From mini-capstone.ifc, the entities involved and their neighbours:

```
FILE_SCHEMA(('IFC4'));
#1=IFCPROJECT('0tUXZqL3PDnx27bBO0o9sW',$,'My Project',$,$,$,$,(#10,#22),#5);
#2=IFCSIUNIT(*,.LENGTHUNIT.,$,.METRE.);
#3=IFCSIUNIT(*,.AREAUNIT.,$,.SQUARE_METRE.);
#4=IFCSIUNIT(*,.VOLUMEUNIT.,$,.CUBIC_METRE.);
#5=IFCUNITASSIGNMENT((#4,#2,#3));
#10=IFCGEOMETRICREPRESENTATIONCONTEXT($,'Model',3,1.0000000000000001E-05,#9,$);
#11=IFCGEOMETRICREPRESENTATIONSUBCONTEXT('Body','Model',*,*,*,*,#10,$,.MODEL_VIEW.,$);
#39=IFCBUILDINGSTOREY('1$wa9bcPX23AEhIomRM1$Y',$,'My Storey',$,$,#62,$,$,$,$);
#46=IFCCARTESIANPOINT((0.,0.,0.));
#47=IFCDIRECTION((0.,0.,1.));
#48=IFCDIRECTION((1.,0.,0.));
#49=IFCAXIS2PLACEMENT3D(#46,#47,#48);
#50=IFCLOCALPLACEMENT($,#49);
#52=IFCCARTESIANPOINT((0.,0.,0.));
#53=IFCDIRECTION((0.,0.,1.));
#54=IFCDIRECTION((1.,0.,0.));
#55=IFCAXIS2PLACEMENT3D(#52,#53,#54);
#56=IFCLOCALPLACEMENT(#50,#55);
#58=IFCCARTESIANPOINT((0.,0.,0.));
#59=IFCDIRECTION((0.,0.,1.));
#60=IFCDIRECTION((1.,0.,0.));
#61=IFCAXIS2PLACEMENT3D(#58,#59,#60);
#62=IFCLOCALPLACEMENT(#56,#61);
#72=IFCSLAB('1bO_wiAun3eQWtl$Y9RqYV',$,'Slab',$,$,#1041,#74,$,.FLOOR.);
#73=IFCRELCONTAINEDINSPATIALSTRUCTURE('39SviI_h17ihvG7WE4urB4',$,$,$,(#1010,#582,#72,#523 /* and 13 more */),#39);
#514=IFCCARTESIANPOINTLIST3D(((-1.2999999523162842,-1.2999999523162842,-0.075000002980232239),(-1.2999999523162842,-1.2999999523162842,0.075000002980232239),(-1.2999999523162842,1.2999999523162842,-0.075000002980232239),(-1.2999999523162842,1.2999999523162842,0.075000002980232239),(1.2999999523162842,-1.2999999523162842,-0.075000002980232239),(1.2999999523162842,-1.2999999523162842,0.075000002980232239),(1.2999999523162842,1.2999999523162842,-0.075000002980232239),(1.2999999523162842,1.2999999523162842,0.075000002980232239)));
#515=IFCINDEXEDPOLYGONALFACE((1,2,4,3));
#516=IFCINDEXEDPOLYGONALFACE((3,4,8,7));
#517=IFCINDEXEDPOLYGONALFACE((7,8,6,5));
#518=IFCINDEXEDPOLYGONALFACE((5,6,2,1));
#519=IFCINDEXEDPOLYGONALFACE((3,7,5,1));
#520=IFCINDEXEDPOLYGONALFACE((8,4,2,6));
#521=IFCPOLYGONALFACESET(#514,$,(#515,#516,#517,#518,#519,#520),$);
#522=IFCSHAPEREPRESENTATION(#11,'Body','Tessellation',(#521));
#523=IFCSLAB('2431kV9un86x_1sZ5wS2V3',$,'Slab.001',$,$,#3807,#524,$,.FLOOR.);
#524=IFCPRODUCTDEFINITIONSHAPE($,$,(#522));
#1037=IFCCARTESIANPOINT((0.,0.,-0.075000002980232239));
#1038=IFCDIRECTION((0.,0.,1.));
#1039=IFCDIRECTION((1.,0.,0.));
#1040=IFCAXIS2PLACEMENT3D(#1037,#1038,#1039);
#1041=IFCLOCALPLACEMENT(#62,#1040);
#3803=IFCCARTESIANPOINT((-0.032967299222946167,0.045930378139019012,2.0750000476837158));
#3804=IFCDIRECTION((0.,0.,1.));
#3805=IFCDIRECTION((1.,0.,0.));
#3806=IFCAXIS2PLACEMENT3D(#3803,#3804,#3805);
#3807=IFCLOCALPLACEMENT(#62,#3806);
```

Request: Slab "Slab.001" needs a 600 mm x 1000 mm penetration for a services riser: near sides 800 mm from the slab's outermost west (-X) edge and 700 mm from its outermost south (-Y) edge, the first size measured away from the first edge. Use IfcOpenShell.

```python
import numpy as np
import ifcopenshell
import ifcopenshell.api.feature
import ifcopenshell.api.geometry
import ifcopenshell.api.root
import ifcopenshell.geom
import ifcopenshell.util.placement
import ifcopenshell.util.representation
import ifcopenshell.util.shape
import ifcopenshell.util.unit

model = ifcopenshell.open("mini-capstone.ifc")
unit_scale = ifcopenshell.util.unit.calculate_unit_scale(model)
settings = ifcopenshell.geom.settings()


def volume(element):
    """Net volume in cubic metres, openings subtracted."""
    shape = ifcopenshell.geom.create_shape(settings, element)
    return ifcopenshell.util.shape.get_volume(shape.geometry)


slab = model.by_guid("2431kV9un86x_1sZ5wS2V3")
before = volume(slab)

# Extent in the slab's own axes, in metres. The edges named are its -X and -Y sides.
slab_shape = ifcopenshell.geom.create_shape(settings, slab)
vertices = ifcopenshell.util.shape.get_vertices(slab_shape.geometry)
x_min, y_min, bottom = vertices.min(axis=0)
top = vertices[:, 2].max()

opening = ifcopenshell.api.root.create_entity(model, ifc_class="IfcOpeningElement", name="Services riser opening", predefined_type="OPENING")
context = ifcopenshell.util.representation.get_context(model, "Model", "Body", "MODEL_VIEW")
width, depth = 0.6, 1
outline = [(0.0, 0.0), (width, 0.0), (width, depth), (0.0, depth), (0.0, 0.0)]
# Overshoot both faces by 50 mm so the cut is clean.
shape = ifcopenshell.api.geometry.add_slab_representation(
    model, context=context, depth=top - bottom + 0.1, polyline=outline
)
ifcopenshell.api.geometry.assign_representation(model, product=opening, representation=shape)

matrix = ifcopenshell.util.placement.get_local_placement(slab.ObjectPlacement)
matrix[:, 3] = matrix @ np.append(np.array([x_min + 0.8, y_min + 0.7, bottom - 0.05]) / unit_scale, 1.0)
ifcopenshell.api.geometry.edit_object_placement(model, product=opening, matrix=matrix, is_si=False)
ifcopenshell.api.feature.add_feature(model, feature=opening, element=slab)

after = volume(slab)

print(f"slab volume {before:.3f} -> {after:.3f} m3")

model.write("mini-capstone_rev.ifc")
```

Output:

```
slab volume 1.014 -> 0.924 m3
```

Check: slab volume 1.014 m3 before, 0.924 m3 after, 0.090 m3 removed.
